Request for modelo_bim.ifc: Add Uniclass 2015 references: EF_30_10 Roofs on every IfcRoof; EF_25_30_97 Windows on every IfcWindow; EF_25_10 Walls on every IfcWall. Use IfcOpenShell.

First a look at what the model holds.

```python
import ifcopenshell

model = ifcopenshell.open("modelo_bim.ifc")
print(model.schema)
print("classifications:", [c.Name for c in model.by_type("IfcClassification")])
for ifc_class in ("IfcDoor", "IfcRoof", "IfcStair", "IfcWall", "IfcWindow"):
    print(ifc_class, len(model.by_type(ifc_class)))
```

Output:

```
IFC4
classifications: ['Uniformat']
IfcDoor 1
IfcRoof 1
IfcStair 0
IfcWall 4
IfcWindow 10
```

```python
import ifcopenshell
import ifcopenshell.api.classification

model = ifcopenshell.open("modelo_bim.ifc")

system = ifcopenshell.api.classification.add_classification(model, classification="Uniclass 2015")

codes = {
    "IfcRoof": ("EF_30_10", "Roofs"),
    "IfcWindow": ("EF_25_30_97", "Windows"),
    "IfcWall": ("EF_25_10", "Walls"),
}
for ifc_class, (code, name) in codes.items():
    products = model.by_type(ifc_class)
    ifcopenshell.api.classification.add_reference(
        model, products=products, classification=system, identification=code, name=name
    )
    print(code, len(products))

model.write("modelo_bim-out.ifc")
```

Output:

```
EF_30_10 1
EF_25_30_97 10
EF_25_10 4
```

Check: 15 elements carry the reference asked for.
